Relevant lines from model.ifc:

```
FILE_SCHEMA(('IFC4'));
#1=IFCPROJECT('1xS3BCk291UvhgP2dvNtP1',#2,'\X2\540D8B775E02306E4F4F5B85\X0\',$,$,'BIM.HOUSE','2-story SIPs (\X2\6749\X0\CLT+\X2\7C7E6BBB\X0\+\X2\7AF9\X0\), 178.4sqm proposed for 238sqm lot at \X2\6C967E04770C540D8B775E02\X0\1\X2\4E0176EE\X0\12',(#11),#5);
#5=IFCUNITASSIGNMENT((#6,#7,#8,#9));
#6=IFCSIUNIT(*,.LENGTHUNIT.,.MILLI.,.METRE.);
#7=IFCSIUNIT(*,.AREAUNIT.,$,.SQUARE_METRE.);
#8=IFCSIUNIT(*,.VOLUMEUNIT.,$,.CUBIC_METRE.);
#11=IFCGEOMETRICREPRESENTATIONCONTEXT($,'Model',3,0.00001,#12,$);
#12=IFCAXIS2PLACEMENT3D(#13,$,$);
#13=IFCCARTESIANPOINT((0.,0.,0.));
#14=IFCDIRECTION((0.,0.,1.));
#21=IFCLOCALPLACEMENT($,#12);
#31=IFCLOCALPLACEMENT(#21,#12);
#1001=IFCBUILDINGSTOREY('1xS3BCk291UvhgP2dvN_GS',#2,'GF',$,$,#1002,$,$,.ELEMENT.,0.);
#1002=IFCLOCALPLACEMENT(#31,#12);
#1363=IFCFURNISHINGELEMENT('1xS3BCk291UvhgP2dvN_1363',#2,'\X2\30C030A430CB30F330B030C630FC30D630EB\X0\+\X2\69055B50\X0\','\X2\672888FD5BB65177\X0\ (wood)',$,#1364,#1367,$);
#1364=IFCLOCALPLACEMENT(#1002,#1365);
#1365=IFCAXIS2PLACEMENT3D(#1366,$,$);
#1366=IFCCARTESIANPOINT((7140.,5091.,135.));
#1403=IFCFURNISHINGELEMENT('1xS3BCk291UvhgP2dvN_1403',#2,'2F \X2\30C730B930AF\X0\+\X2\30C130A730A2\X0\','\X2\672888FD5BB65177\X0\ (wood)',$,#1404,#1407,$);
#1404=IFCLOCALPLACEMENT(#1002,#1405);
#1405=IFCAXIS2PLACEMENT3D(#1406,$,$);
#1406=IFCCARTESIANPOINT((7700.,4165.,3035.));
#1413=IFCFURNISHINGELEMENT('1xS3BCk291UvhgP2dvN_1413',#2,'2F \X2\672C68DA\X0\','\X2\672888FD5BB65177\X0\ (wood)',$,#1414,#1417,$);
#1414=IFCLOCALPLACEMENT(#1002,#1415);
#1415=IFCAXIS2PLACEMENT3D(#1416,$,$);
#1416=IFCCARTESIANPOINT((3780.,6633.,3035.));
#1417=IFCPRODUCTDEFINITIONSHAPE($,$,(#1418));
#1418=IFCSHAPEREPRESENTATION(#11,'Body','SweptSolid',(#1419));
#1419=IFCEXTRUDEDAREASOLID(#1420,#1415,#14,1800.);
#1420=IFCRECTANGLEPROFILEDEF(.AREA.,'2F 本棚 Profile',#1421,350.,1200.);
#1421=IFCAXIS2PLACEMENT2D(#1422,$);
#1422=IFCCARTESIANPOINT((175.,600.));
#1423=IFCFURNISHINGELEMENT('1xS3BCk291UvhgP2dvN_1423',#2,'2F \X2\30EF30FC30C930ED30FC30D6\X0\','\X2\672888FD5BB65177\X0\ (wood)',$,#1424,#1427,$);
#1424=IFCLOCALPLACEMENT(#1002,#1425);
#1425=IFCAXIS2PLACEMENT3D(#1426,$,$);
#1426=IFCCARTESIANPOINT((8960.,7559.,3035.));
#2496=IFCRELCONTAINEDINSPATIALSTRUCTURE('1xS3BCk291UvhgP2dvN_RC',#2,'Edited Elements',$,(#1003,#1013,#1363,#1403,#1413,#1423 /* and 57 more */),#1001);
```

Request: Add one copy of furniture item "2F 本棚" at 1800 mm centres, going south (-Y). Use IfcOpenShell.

```python
import numpy as np
import ifcopenshell
import ifcopenshell.api.geometry
import ifcopenshell.api.root
import ifcopenshell.util.element
import ifcopenshell.util.placement
import ifcopenshell.util.unit

model = ifcopenshell.open("model.ifc")
unit_scale = ifcopenshell.util.unit.calculate_unit_scale(model)


def reuse_history(source, copy):
    """copy_class also copies each property set's owner history, people and application; keep the originals."""
    for rel in copy.IsDefinedBy:
        if rel.is_a("IfcRelDefinesByProperties") and (history := rel.RelatingPropertyDefinition.OwnerHistory):
            rel.RelatingPropertyDefinition.OwnerHistory = source.OwnerHistory
            ifcopenshell.util.element.remove_deep2(model, history)


source = model.by_id(1413)
base = ifcopenshell.util.placement.get_local_placement(source.ObjectPlacement)
step = np.array([0.0, -1.0, 0.0]) * 1.8 / unit_scale

for i in range(1, 2):
    copy = ifcopenshell.api.root.copy_class(model, product=source)
    copy.Representation = ifcopenshell.util.element.copy_deep(
        model, source.Representation, exclude=["IfcGeometricRepresentationContext", "IfcRepresentationMap"]
    )
    reuse_history(source, copy)
    matrix = base.copy()
    matrix[:3, 3] += i * step
    print("added at", matrix[:3, 3].round(3) + 0.0)
    ifcopenshell.api.geometry.edit_object_placement(model, product=copy, matrix=matrix, is_si=False)

model.write("model_v2.ifc")
```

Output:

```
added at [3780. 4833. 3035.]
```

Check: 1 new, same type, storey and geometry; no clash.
